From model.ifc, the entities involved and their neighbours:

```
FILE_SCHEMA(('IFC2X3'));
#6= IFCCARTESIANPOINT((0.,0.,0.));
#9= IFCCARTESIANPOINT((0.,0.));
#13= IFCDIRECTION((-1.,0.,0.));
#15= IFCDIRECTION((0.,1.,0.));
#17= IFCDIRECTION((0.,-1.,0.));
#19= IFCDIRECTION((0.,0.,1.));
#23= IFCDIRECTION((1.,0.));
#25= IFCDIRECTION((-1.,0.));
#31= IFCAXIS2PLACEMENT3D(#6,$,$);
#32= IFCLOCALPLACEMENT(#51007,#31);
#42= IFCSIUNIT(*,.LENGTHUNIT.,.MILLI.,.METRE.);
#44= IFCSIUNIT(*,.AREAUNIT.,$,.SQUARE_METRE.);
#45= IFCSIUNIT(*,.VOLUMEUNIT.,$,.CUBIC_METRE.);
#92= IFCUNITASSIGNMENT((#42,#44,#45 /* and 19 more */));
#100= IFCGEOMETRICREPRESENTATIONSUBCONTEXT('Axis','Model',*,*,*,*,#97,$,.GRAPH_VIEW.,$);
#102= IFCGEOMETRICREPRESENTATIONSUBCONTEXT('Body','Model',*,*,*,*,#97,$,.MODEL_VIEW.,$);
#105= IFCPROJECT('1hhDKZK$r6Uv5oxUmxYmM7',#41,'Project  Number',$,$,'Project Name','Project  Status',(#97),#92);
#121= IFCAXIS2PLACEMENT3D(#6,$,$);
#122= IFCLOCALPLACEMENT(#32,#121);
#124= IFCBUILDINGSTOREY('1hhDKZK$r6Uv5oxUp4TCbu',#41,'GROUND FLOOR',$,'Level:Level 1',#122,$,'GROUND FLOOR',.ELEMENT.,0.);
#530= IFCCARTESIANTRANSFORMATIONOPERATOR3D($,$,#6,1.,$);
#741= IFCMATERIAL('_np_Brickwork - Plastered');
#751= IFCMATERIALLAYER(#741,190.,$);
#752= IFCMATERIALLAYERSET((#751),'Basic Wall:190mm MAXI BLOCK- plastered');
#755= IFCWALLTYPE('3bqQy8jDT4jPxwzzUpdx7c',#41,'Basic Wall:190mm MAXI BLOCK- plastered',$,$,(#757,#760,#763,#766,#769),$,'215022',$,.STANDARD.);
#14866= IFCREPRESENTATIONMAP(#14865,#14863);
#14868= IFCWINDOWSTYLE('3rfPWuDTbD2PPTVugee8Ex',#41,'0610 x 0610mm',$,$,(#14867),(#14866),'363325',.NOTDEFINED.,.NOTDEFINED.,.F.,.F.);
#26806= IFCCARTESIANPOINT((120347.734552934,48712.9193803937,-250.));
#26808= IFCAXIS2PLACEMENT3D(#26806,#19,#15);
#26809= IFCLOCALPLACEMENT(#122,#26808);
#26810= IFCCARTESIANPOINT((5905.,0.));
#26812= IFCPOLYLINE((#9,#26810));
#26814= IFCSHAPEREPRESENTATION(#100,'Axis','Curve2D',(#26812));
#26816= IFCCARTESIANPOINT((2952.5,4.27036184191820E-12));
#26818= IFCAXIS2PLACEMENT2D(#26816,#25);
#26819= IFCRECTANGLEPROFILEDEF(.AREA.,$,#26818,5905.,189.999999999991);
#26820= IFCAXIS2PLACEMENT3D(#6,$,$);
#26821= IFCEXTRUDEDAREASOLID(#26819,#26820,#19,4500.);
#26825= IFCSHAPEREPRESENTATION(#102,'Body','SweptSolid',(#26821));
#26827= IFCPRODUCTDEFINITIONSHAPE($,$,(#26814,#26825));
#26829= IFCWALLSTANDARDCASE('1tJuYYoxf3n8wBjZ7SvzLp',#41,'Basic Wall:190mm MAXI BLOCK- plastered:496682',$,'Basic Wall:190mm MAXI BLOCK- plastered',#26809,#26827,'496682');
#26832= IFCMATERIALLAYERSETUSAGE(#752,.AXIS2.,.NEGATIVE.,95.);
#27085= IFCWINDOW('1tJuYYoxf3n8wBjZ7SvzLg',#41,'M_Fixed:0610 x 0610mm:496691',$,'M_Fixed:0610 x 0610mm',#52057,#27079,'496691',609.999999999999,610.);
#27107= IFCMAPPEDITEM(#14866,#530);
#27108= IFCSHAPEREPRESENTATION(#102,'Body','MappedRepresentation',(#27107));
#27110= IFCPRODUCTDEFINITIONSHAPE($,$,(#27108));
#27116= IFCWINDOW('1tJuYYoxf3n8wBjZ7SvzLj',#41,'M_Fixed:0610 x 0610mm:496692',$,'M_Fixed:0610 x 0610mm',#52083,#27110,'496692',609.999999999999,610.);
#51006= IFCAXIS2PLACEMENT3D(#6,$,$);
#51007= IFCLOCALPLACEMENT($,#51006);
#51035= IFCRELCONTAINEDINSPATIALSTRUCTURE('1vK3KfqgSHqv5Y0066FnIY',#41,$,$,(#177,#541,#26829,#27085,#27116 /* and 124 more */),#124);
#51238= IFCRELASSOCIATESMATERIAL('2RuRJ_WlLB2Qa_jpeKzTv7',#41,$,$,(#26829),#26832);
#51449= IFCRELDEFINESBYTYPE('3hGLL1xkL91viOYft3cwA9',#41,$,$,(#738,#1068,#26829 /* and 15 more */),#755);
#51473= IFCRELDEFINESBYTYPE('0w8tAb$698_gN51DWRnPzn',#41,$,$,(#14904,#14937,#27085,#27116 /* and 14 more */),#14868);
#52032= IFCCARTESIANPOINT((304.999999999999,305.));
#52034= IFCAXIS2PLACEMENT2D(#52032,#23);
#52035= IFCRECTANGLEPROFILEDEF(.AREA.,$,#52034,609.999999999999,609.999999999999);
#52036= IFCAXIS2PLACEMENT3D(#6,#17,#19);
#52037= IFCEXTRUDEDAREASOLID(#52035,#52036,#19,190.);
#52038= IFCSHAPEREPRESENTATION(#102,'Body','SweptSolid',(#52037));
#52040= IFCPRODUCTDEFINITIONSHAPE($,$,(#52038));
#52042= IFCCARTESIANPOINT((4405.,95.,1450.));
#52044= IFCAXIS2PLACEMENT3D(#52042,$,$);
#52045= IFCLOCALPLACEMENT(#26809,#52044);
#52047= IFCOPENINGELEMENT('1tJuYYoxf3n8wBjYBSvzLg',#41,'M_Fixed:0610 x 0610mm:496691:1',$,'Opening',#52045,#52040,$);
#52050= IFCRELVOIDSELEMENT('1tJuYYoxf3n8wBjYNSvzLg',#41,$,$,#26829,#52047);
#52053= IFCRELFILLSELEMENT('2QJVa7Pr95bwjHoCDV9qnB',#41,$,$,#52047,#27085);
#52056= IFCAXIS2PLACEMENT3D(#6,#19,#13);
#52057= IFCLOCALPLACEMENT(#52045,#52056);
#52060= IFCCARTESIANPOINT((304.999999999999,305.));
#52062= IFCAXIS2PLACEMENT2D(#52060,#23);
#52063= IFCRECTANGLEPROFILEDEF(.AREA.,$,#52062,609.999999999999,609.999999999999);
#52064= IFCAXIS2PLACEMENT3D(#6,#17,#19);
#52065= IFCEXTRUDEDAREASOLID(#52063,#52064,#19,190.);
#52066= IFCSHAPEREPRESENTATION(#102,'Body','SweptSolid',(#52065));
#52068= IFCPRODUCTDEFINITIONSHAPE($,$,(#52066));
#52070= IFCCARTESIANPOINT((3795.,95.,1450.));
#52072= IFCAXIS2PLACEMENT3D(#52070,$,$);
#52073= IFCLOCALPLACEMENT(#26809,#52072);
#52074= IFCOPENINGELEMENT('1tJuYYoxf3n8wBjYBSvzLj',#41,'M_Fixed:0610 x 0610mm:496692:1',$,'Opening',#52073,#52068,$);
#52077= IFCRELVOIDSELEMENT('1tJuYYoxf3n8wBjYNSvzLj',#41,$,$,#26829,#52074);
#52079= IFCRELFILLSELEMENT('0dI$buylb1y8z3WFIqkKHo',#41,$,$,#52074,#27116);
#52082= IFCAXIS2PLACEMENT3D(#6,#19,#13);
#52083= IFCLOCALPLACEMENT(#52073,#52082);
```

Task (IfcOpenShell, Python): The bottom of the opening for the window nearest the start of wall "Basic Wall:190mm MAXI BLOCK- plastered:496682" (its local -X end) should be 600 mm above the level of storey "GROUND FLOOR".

```python
import numpy as np
import ifcopenshell
import ifcopenshell.api.geometry
import ifcopenshell.geom
import ifcopenshell.util.element
import ifcopenshell.util.placement
import ifcopenshell.util.shape
import ifcopenshell.util.unit

model = ifcopenshell.open("model.ifc")
unit_scale = ifcopenshell.util.unit.calculate_unit_scale(model)

window = model.by_id(27116)
opening = window.FillsVoids[0].RelatingOpeningElement
storey = ifcopenshell.util.element.get_container(window, ifc_class="IfcBuildingStorey")
level = ifcopenshell.util.placement.get_local_placement(storey.ObjectPlacement)[2, 3]

# The opening's origin need not be at the sill, so measure its lowest point.
shape = ifcopenshell.geom.create_shape(ifcopenshell.geom.settings(), opening)
bottom = ifcopenshell.util.shape.get_shape_bottom_elevation(shape, shape.geometry) / unit_scale
dz = level + 0.6 / unit_scale - bottom

shift = np.array([0.0, 0.0, dz])
# The window is placed relative to its opening, so it follows when the opening moves.
matrix = ifcopenshell.util.placement.get_local_placement(opening.ObjectPlacement)
matrix[:3, 3] += shift
ifcopenshell.api.geometry.edit_object_placement(
    model, product=opening, matrix=matrix, is_si=False, should_transform_children=True
)

print(f"moved by {dz * unit_scale:+.3f} m")

model.write("model_updated.ifc")
```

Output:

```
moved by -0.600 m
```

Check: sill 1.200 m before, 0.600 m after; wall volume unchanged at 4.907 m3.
